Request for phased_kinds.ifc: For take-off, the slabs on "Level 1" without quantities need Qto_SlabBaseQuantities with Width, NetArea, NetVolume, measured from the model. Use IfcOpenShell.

First a look at what the model holds.

```python
import ifcopenshell
import ifcopenshell.util.element
import ifcopenshell.util.unit

model = ifcopenshell.open("phased_kinds.ifc")
print(model.schema)
for unit_type in ("LENGTHUNIT", "AREAUNIT", "VOLUMEUNIT"):
    print(unit_type, ifcopenshell.util.unit.calculate_unit_scale(model, unit_type))
storey = next(s for s in model.by_type("IfcBuildingStorey") if s.Name == "Level 1")
slabs = [e for e in ifcopenshell.util.element.get_decomposition(storey) if e.is_a("IfcSlab")]
for e in sorted(slabs, key=lambda e: e.id()):
    print(e.id(), e.is_a(), e.Name, list(ifcopenshell.util.element.get_psets(e, qtos_only=True)), sep=" | ")
```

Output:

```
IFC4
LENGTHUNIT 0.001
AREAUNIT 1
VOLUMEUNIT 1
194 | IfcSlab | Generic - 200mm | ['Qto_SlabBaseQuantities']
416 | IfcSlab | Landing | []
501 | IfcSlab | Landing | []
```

```python
import ifcopenshell
import ifcopenshell.api.pset
import ifcopenshell.geom
import ifcopenshell.util.element
import ifcopenshell.util.shape
import ifcopenshell.util.unit

model = ifcopenshell.open("phased_kinds.ifc")
unit_scale = ifcopenshell.util.unit.calculate_unit_scale(model)
area_scale = ifcopenshell.util.unit.calculate_unit_scale(model, "AREAUNIT")
volume_scale = ifcopenshell.util.unit.calculate_unit_scale(model, "VOLUMEUNIT")
settings = ifcopenshell.geom.settings()

storey = next(s for s in model.by_type("IfcBuildingStorey") if s.Name == "Level 1")
slabs = [e for e in ifcopenshell.util.element.get_decomposition(storey) if e.is_a("IfcSlab")]

for e in sorted(slabs, key=lambda e: e.id()):
    if ifcopenshell.util.element.get_psets(e, qtos_only=True, should_inherit=False):
        continue
    # Geometry comes back in metres, in the element's own axes.
    shape = ifcopenshell.geom.create_shape(settings, e)
    values = {
        "Width": ifcopenshell.util.shape.get_z(shape.geometry) / unit_scale,
        "NetArea": ifcopenshell.util.shape.get_footprint_area(shape.geometry) / area_scale,
        "NetVolume": ifcopenshell.util.shape.get_volume(shape.geometry) / volume_scale,
    }
    qto = ifcopenshell.api.pset.add_qto(model, product=e, name="Qto_SlabBaseQuantities")
    ifcopenshell.api.pset.edit_qto(model, qto=qto, properties=values)
    print(e.id(), {k: round(v, 3) for k, v in values.items()})

model.write("phased_kinds_v2.ifc")
```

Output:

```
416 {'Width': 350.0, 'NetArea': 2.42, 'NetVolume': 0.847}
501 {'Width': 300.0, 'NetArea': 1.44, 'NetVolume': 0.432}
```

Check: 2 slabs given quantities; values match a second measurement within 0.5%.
